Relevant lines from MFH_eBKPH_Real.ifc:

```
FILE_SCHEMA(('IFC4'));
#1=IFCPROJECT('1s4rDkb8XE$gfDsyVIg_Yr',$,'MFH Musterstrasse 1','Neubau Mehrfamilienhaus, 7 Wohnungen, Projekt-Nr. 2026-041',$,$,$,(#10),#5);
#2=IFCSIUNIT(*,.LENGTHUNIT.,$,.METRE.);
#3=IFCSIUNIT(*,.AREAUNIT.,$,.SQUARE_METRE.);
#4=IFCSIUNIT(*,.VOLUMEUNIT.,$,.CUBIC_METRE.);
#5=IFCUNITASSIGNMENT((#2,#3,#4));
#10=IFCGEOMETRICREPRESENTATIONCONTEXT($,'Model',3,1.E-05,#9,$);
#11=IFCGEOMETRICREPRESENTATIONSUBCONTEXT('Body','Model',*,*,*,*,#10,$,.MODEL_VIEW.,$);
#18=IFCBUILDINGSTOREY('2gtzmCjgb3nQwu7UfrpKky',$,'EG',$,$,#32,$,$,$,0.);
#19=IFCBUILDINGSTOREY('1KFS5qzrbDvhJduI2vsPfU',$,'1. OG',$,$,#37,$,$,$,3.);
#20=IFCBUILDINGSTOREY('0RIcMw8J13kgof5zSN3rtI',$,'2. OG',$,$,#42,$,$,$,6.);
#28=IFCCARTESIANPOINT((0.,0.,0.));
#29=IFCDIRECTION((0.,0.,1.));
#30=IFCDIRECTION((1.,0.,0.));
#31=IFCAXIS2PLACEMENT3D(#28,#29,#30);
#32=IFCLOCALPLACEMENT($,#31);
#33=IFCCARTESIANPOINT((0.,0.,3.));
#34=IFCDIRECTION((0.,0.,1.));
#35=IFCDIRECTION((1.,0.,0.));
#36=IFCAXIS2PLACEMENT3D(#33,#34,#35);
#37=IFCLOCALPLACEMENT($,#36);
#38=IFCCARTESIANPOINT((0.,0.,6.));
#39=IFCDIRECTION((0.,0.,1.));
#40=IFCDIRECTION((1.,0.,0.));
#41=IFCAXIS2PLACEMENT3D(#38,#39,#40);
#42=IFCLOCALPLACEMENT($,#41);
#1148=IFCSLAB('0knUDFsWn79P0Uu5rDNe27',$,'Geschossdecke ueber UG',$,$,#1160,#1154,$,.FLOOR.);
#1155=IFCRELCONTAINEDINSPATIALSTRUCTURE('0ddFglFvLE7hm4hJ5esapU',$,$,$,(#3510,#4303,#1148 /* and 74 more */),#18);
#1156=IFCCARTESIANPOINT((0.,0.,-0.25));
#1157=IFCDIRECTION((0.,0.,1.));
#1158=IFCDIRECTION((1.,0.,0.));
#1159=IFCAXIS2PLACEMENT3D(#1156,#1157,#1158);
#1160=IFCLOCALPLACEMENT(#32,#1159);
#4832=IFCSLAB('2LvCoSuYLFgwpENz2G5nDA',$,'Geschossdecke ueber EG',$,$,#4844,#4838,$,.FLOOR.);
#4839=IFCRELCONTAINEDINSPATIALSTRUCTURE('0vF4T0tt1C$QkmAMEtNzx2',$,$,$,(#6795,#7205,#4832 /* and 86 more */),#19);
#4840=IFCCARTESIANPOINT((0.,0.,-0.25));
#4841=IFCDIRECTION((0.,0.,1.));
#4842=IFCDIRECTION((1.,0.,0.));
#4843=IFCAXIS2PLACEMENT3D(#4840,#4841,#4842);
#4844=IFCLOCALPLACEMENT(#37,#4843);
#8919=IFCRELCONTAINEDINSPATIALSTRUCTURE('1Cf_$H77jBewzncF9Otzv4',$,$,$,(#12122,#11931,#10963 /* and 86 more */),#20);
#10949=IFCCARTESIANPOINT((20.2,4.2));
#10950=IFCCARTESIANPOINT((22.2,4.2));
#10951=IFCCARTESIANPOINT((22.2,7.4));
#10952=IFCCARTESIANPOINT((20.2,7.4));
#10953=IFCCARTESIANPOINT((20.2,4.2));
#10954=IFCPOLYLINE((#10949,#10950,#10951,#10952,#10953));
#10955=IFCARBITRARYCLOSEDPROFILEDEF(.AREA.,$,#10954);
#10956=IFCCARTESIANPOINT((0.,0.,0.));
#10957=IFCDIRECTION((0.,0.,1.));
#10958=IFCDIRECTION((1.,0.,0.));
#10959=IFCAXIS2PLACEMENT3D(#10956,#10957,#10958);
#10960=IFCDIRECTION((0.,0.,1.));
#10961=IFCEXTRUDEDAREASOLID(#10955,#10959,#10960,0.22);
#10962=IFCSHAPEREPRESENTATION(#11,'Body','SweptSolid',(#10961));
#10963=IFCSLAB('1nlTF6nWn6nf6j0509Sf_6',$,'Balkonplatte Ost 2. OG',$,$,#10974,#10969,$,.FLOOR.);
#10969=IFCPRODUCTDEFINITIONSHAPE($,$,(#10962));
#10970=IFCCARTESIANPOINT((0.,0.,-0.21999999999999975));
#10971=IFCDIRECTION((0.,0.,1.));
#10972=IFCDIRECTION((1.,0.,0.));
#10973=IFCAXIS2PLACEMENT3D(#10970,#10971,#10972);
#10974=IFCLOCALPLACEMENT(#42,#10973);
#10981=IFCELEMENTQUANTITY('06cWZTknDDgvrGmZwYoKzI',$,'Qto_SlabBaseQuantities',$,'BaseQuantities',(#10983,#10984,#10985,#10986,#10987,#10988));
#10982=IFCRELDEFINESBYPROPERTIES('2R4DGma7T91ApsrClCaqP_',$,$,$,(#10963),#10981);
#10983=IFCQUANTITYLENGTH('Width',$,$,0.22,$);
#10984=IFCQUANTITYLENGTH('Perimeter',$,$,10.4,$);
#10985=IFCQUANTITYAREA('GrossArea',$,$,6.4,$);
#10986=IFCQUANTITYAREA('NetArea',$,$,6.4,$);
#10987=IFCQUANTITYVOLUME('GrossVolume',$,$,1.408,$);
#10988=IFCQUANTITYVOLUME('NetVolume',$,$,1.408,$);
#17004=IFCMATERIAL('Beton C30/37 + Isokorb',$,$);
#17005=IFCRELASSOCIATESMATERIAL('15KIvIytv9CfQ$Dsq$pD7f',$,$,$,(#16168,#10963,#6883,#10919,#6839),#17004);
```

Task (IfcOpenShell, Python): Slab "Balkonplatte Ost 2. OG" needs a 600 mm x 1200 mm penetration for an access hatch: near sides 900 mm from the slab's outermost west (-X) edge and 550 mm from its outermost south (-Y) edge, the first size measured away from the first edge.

```python
import numpy as np
import ifcopenshell
import ifcopenshell.api.feature
import ifcopenshell.api.geometry
import ifcopenshell.api.pset
import ifcopenshell.api.root
import ifcopenshell.geom
import ifcopenshell.util.element
import ifcopenshell.util.placement
import ifcopenshell.util.representation
import ifcopenshell.util.shape
import ifcopenshell.util.unit

model = ifcopenshell.open("MFH_eBKPH_Real.ifc")
unit_scale = ifcopenshell.util.unit.calculate_unit_scale(model)
area_scale = ifcopenshell.util.unit.calculate_unit_scale(model, "AREAUNIT")
volume_scale = ifcopenshell.util.unit.calculate_unit_scale(model, "VOLUMEUNIT")
settings = ifcopenshell.geom.settings()


def volume(element):
    """Net volume in cubic metres, openings subtracted."""
    shape = ifcopenshell.geom.create_shape(settings, element)
    return ifcopenshell.util.shape.get_volume(shape.geometry)


slab = model.by_guid("1nlTF6nWn6nf6j0509Sf_6")
before = volume(slab)

# Extent in the slab's own axes, in metres. The edges named are its -X and -Y sides.
slab_shape = ifcopenshell.geom.create_shape(settings, slab)
vertices = ifcopenshell.util.shape.get_vertices(slab_shape.geometry)
x_min, y_min, bottom = vertices.min(axis=0)
top = vertices[:, 2].max()

opening = ifcopenshell.api.root.create_entity(model, ifc_class="IfcOpeningElement", name="Access hatch opening", predefined_type="OPENING")
context = ifcopenshell.util.representation.get_context(model, "Model", "Body", "MODEL_VIEW")
width, depth = 0.6, 1.2
outline = [(0.0, 0.0), (width, 0.0), (width, depth), (0.0, depth), (0.0, 0.0)]
# Overshoot both faces by 50 mm so the cut is clean.
shape = ifcopenshell.api.geometry.add_slab_representation(
    model, context=context, depth=top - bottom + 0.1, polyline=outline
)
ifcopenshell.api.geometry.assign_representation(model, product=opening, representation=shape)

matrix = ifcopenshell.util.placement.get_local_placement(slab.ObjectPlacement)
matrix[:, 3] = matrix @ np.append(np.array([x_min + 0.9, y_min + 0.55, bottom - 0.05]) / unit_scale, 1.0)
ifcopenshell.api.geometry.edit_object_placement(model, product=opening, matrix=matrix, is_si=False)
ifcopenshell.api.feature.add_feature(model, feature=opening, element=slab)

after = volume(slab)

# Update the slab's stored quantities.
qto = model.by_id(ifcopenshell.util.element.get_pset(slab, "Qto_SlabBaseQuantities", should_inherit=False)["id"])
ifcopenshell.api.pset.edit_qto(model, qto=qto, properties={
    "NetArea": after / (top - bottom) / area_scale,
    "NetVolume": after / volume_scale,
})

print(f"slab volume {before:.3f} -> {after:.3f} m3")

model.write("MFH_eBKPH_Real_v2.ifc")
```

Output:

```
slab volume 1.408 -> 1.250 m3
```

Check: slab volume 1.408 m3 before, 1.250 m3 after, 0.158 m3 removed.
